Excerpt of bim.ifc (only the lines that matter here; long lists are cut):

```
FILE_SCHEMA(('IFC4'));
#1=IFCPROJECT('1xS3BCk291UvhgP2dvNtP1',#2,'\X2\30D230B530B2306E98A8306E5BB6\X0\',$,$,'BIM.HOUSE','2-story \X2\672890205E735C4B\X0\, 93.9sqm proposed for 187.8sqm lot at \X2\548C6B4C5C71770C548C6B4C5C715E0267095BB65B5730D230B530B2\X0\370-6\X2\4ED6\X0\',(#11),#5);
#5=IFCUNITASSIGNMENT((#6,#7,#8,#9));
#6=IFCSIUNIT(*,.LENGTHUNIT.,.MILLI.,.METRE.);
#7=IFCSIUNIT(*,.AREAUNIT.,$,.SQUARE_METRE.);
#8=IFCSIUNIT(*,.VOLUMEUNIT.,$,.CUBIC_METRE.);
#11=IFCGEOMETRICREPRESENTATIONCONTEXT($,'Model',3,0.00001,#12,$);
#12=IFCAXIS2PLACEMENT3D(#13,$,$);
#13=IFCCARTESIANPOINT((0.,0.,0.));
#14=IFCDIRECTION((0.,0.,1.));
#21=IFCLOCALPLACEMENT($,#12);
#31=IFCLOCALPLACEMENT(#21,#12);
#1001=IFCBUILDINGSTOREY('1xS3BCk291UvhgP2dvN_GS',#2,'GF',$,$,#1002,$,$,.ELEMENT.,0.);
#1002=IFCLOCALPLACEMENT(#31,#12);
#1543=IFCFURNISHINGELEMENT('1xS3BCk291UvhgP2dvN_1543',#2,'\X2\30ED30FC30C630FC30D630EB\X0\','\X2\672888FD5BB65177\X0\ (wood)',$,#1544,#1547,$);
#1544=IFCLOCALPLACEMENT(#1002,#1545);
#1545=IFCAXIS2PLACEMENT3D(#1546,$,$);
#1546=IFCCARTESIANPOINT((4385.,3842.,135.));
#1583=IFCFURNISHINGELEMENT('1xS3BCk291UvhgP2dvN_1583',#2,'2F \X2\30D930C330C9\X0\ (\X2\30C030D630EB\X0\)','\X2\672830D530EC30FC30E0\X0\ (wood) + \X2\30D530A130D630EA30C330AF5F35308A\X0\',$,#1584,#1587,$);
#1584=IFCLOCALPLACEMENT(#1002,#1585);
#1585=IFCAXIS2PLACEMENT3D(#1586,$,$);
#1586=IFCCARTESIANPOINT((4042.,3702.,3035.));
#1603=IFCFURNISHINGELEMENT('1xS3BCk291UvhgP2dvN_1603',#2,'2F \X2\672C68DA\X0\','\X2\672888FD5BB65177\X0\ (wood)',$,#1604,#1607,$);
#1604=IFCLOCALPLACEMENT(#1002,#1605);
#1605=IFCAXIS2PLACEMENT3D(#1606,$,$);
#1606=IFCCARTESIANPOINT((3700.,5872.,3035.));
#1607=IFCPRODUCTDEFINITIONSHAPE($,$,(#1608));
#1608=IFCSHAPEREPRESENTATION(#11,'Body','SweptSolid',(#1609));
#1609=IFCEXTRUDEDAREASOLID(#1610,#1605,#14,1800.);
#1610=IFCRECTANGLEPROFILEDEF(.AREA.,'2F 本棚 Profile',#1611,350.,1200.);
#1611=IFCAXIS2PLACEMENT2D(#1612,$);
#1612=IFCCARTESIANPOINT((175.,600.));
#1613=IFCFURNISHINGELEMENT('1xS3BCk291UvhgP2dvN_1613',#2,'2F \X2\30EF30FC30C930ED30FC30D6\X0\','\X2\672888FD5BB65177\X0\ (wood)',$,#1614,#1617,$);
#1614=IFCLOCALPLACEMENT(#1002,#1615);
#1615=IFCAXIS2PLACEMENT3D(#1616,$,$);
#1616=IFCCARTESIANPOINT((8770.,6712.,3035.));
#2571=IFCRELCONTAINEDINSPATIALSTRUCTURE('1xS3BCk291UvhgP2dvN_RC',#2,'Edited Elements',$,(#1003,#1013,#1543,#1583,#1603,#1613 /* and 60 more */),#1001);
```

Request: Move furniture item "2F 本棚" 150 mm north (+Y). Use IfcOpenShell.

```python
import ifcopenshell
import ifcopenshell.api.geometry
import ifcopenshell.util.placement
import ifcopenshell.util.unit

model = ifcopenshell.open("bim.ifc")
unit_scale = ifcopenshell.util.unit.calculate_unit_scale(model)

item = model.by_id(1603)
matrix = ifcopenshell.util.placement.get_local_placement(item.ObjectPlacement)
matrix[1, 3] += 0.15 / unit_scale
ifcopenshell.api.geometry.edit_object_placement(model, product=item, matrix=matrix, is_si=False)

print(ifcopenshell.util.placement.get_local_placement(item.ObjectPlacement).round(3) + 0.0)

model.write("bim-out.ifc")
```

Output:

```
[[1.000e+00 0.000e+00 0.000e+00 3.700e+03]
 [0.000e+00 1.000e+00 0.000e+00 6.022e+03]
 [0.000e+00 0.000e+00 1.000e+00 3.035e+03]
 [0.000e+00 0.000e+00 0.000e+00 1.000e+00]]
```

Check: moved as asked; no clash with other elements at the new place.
